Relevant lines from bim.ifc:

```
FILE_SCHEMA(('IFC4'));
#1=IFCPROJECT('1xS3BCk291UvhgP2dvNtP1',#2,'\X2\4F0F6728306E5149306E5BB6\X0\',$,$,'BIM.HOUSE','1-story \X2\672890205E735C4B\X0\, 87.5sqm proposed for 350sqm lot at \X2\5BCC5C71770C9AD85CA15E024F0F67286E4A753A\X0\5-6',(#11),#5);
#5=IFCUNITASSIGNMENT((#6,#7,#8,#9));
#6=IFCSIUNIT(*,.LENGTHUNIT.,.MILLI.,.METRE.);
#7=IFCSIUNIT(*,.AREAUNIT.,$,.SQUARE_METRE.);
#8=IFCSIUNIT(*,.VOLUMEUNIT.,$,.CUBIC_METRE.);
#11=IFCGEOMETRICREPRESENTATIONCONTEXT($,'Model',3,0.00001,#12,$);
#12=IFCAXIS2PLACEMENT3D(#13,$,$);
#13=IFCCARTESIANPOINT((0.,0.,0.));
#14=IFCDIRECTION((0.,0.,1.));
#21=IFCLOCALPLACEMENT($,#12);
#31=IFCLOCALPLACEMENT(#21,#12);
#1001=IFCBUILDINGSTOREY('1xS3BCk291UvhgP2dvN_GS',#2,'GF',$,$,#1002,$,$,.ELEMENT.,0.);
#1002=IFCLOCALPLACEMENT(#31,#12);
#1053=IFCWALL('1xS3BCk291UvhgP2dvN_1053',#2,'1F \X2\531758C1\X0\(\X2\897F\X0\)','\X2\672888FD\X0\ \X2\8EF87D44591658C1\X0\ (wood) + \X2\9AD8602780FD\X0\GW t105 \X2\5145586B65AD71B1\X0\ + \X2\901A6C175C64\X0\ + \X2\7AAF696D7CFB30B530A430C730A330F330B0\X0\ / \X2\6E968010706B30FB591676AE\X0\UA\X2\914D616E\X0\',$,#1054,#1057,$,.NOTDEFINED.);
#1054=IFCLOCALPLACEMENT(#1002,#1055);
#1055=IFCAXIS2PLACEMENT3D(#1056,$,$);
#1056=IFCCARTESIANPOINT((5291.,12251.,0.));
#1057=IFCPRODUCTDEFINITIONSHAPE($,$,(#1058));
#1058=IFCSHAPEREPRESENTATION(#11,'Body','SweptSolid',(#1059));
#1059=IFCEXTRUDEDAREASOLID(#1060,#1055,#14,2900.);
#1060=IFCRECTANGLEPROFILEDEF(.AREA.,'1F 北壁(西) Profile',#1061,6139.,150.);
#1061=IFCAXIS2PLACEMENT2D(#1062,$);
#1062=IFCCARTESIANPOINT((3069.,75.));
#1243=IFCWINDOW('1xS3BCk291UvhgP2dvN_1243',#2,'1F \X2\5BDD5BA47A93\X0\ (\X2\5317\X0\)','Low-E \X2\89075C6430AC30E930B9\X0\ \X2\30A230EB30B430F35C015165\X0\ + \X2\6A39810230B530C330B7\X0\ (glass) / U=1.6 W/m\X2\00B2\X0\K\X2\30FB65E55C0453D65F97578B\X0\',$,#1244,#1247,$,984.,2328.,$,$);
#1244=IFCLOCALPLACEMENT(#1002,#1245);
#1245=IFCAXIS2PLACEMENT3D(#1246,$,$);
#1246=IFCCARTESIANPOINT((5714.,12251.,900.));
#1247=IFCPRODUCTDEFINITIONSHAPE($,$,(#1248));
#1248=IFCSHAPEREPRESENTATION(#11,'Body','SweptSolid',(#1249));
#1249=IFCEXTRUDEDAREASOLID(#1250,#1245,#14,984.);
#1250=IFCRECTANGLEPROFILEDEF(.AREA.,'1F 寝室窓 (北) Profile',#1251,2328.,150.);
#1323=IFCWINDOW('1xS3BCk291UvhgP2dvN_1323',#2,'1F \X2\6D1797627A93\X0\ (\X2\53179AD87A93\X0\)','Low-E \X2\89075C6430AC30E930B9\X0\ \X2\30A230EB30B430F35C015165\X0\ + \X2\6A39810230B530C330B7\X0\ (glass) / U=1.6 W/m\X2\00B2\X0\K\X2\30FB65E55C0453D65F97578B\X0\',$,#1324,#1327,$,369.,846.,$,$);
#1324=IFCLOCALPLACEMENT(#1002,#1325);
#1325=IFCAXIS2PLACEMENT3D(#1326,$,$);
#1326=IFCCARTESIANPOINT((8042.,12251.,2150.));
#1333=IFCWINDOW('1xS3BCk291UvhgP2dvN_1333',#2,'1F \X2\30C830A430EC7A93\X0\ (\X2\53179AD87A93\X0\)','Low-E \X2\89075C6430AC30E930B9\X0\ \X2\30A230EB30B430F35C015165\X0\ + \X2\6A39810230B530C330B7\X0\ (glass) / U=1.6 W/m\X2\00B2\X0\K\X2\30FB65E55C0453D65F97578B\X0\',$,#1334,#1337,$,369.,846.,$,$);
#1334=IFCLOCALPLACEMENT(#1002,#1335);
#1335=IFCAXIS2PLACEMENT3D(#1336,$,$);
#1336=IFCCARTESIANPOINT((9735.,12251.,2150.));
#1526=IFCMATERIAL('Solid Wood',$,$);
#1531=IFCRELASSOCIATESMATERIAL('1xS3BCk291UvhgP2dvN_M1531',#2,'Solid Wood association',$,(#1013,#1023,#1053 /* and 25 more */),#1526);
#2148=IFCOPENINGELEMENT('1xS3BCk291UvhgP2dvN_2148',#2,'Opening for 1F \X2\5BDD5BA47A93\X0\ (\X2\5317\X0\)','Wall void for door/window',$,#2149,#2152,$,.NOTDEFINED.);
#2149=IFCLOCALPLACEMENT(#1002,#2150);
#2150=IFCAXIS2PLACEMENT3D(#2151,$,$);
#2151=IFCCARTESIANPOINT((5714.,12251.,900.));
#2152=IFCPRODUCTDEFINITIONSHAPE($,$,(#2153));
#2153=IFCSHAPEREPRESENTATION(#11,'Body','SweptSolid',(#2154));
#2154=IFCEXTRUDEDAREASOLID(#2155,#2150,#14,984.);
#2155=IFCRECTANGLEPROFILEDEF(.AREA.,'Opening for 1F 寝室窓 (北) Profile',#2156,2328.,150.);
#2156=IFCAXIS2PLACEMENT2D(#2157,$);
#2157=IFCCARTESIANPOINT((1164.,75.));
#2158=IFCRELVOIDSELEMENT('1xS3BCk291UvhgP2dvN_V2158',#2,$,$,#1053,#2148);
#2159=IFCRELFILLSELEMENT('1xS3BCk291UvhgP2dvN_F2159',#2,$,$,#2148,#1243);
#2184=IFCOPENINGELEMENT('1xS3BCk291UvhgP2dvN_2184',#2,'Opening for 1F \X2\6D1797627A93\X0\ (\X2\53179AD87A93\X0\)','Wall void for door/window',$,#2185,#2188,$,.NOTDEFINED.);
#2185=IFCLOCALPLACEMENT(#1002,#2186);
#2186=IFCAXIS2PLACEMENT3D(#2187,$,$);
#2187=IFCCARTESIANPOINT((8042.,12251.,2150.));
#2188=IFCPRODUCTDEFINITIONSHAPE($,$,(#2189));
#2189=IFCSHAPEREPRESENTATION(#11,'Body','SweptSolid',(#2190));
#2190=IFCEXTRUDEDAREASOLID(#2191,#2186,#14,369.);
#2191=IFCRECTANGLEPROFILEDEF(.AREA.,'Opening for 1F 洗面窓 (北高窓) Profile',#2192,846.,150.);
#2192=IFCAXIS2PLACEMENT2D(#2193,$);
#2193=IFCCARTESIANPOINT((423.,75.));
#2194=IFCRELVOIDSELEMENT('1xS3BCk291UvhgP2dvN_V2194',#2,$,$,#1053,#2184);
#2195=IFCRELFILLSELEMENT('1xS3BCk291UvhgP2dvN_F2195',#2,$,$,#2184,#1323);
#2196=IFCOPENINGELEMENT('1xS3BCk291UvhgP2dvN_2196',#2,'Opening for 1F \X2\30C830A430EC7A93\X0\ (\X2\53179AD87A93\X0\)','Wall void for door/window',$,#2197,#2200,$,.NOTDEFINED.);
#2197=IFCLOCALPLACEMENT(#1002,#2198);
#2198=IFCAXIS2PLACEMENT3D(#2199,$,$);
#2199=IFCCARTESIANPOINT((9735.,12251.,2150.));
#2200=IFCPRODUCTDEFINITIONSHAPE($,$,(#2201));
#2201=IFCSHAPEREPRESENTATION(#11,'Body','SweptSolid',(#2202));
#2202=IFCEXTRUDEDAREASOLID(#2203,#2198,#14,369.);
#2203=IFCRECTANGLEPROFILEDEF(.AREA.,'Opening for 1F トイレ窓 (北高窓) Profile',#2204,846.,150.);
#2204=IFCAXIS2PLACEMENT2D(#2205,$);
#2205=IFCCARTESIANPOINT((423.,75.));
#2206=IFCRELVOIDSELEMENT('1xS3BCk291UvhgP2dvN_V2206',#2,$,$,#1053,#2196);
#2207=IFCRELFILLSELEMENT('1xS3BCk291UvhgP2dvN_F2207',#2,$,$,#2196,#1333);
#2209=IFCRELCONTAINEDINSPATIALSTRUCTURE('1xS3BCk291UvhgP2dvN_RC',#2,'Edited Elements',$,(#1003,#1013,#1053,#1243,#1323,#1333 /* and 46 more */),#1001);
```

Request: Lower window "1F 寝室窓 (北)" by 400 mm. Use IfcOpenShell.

```python
import numpy as np
import ifcopenshell
import ifcopenshell.api.geometry
import ifcopenshell.util.placement
import ifcopenshell.util.unit

model = ifcopenshell.open("bim.ifc")
unit_scale = ifcopenshell.util.unit.calculate_unit_scale(model)

window = model.by_guid("1xS3BCk291UvhgP2dvN_1243")
opening = window.FillsVoids[0].RelatingOpeningElement
dz = -0.4 / unit_scale

shift = np.array([0.0, 0.0, dz])
# The window is not placed relative to its opening, so move both.
for product in (opening, window):
    matrix = ifcopenshell.util.placement.get_local_placement(product.ObjectPlacement)
    matrix[:3, 3] += shift
    ifcopenshell.api.geometry.edit_object_placement(model, product=product, matrix=matrix, is_si=False)

print(f"moved by {dz * unit_scale:+.3f} m")

model.write("bim_edited.ifc")
```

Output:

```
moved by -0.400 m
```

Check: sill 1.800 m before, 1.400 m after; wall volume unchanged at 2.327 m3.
